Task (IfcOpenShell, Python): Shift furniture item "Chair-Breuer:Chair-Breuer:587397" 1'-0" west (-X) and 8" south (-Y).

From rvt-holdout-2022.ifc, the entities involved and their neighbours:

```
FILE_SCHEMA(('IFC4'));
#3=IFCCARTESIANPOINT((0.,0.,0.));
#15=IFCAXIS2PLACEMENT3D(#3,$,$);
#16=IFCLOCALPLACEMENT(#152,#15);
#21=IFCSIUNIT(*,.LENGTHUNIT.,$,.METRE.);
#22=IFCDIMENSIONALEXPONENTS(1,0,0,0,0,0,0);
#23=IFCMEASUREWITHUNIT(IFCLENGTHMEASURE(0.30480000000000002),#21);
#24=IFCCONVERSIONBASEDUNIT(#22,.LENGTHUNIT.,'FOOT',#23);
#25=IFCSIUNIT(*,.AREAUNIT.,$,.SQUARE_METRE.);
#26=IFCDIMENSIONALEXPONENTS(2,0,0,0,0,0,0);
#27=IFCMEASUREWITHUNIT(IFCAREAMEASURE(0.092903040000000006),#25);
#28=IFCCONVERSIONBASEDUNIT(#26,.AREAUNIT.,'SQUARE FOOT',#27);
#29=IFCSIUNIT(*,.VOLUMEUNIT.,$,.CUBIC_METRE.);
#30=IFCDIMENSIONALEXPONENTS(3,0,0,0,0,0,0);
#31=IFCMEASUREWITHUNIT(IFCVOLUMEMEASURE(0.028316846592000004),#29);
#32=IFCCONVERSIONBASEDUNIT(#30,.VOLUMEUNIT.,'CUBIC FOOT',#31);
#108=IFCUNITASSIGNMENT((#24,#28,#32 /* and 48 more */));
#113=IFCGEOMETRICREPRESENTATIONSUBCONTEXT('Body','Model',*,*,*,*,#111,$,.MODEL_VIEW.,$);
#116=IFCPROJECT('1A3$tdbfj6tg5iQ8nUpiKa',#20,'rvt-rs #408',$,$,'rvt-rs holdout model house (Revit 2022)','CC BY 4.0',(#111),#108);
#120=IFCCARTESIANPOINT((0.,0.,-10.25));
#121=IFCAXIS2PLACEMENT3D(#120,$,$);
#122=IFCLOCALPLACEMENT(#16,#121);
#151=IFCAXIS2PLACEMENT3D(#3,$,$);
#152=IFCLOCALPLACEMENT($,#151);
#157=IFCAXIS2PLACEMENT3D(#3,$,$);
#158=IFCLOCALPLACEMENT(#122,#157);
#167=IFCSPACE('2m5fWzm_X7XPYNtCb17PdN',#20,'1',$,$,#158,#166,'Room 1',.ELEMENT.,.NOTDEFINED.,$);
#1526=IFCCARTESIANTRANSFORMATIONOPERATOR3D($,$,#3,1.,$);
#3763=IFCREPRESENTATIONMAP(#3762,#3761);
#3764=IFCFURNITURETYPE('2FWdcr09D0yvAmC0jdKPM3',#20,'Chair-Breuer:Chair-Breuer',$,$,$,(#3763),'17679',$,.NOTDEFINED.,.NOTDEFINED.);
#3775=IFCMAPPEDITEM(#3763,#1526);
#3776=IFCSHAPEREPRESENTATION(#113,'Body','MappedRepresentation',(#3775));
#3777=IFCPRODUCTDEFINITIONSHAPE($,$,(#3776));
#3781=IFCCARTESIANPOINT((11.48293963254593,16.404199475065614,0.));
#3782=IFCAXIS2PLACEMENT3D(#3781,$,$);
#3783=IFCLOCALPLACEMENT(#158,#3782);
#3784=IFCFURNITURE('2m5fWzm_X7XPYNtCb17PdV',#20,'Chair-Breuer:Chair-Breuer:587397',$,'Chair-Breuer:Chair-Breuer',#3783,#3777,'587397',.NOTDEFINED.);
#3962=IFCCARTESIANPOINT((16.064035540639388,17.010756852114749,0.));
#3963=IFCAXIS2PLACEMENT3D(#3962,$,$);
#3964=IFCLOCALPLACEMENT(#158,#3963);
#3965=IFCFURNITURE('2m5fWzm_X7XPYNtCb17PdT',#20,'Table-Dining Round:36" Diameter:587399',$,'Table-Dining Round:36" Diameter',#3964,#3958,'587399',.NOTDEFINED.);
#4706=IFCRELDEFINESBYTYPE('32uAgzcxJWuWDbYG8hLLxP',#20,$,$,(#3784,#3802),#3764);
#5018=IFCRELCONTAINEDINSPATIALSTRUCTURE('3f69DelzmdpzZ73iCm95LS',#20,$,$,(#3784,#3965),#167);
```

```python
import ifcopenshell
import ifcopenshell.api.geometry
import ifcopenshell.util.placement
import ifcopenshell.util.unit

model = ifcopenshell.open("rvt-holdout-2022.ifc")
unit_scale = ifcopenshell.util.unit.calculate_unit_scale(model)

item = model.by_id(3784)
matrix = ifcopenshell.util.placement.get_local_placement(item.ObjectPlacement)
matrix[0, 3] -= 12 * 0.0254 / unit_scale
matrix[1, 3] -= 8 * 0.0254 / unit_scale
ifcopenshell.api.geometry.edit_object_placement(model, product=item, matrix=matrix, is_si=False)

print(ifcopenshell.util.placement.get_local_placement(item.ObjectPlacement).round(3) + 0.0)

model.write("rvt-holdout-2022_updated.ifc")
```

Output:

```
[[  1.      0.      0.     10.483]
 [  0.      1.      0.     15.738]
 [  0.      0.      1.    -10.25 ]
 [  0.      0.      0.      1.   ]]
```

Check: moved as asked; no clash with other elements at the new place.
